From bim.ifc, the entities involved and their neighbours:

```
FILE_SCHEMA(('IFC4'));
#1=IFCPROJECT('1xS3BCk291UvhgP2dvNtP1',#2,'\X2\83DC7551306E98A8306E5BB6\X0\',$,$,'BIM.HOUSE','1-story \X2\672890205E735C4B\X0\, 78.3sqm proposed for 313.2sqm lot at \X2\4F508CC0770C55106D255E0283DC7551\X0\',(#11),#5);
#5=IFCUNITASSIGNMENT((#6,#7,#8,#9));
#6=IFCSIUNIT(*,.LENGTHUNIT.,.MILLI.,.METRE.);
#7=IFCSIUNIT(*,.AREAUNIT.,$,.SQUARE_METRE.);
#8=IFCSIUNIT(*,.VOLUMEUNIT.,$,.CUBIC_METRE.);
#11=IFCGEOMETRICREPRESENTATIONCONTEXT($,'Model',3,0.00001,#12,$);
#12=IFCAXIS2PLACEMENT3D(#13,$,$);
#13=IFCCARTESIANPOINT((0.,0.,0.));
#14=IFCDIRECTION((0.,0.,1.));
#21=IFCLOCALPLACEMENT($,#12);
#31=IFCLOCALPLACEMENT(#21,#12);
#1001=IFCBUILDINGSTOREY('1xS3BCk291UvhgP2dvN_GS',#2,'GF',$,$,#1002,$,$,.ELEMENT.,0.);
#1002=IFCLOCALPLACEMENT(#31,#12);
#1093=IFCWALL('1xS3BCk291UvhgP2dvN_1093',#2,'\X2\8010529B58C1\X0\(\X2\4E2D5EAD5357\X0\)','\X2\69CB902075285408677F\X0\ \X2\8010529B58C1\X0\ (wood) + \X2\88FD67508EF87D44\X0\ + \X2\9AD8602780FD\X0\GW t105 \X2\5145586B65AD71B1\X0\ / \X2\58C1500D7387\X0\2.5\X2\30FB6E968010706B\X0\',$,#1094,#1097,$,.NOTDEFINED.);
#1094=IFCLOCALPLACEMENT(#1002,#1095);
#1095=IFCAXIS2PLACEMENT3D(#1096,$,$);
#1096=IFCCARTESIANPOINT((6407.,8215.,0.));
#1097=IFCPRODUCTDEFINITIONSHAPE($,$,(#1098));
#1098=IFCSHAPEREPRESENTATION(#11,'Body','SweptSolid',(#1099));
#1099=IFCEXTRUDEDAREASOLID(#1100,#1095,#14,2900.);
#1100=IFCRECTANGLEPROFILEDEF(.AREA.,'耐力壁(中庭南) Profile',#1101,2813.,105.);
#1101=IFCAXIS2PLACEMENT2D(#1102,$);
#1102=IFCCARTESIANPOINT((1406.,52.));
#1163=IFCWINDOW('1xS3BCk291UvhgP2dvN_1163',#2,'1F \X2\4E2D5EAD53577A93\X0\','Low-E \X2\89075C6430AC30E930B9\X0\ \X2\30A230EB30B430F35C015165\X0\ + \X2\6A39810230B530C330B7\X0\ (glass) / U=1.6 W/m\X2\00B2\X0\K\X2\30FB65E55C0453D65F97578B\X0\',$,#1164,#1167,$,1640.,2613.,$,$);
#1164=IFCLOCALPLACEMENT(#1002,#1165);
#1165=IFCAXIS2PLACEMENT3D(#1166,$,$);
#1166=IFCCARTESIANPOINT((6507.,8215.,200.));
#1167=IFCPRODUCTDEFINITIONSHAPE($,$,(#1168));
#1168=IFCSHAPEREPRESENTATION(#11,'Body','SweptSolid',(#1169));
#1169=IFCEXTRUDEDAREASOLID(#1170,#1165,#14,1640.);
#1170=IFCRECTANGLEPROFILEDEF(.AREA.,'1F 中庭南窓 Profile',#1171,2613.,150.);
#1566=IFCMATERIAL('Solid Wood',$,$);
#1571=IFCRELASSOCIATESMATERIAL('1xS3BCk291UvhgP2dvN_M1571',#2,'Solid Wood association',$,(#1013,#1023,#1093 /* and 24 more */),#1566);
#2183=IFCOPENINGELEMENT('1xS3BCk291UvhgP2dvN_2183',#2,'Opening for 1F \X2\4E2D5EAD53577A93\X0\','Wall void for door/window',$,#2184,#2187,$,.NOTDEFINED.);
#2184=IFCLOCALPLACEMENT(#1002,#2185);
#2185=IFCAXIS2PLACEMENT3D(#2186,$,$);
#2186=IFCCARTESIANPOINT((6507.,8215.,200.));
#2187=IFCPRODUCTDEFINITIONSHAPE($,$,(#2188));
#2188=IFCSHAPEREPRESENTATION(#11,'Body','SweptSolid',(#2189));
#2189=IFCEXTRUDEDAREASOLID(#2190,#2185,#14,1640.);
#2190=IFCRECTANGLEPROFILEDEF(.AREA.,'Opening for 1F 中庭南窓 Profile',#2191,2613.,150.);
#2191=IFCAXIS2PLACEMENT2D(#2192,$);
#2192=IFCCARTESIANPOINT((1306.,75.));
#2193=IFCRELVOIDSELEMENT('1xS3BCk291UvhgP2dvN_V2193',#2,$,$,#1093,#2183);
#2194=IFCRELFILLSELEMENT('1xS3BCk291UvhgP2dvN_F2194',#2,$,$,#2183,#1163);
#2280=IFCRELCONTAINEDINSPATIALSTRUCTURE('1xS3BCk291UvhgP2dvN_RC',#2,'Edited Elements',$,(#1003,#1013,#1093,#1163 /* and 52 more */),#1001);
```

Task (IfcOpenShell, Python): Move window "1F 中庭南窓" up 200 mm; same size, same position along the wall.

```python
import numpy as np
import ifcopenshell
import ifcopenshell.api.geometry
import ifcopenshell.util.placement
import ifcopenshell.util.unit

model = ifcopenshell.open("bim.ifc")
unit_scale = ifcopenshell.util.unit.calculate_unit_scale(model)

window = model.by_id(1163)
opening = window.FillsVoids[0].RelatingOpeningElement
dz = 0.2 / unit_scale

shift = np.array([0.0, 0.0, dz])
# The window is not placed relative to its opening, so move both.
for product in (opening, window):
    matrix = ifcopenshell.util.placement.get_local_placement(product.ObjectPlacement)
    matrix[:3, 3] += shift
    ifcopenshell.api.geometry.edit_object_placement(model, product=product, matrix=matrix, is_si=False)

print(f"moved by {dz * unit_scale:+.3f} m")

model.write("bim_v2.ifc")
```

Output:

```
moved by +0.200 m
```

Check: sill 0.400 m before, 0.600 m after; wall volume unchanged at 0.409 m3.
